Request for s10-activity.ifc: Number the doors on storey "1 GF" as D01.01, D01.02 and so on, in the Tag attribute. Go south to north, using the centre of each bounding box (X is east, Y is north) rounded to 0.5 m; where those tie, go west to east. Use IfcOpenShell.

First a look at what the model holds.

```python
import ifcopenshell
import ifcopenshell.util.element
import ifcopenshell.util.placement

model = ifcopenshell.open("s10-activity.ifc")
print(model.schema)
storey = next(s for s in model.by_type("IfcBuildingStorey") if s.Name == "1 GF")
doors = [e for e in ifcopenshell.util.element.get_decomposition(storey) if e.is_a("IfcDoor")]
for e in sorted(doors, key=lambda e: e.id()):
    origin = ifcopenshell.util.placement.get_local_placement(e.ObjectPlacement)[:3, 3]
    print(e.id(), e.Tag, e.Name, origin.round(2) + 0.0, sep=" | ")
```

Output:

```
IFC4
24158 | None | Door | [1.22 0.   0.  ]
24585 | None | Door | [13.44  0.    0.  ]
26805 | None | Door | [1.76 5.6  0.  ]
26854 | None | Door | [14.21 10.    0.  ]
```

```python
import ifcopenshell
import ifcopenshell.geom
import ifcopenshell.util.element
import ifcopenshell.util.shape

model = ifcopenshell.open("s10-activity.ifc")
settings = ifcopenshell.geom.settings()
settings.set("use-world-coords", True)


def centre(element):
    shape = ifcopenshell.geom.create_shape(settings, element)
    return ifcopenshell.util.shape.get_bbox_centroid(shape.geometry)


storey = next(s for s in model.by_type("IfcBuildingStorey") if s.Name == "1 GF")
doors = [e for e in ifcopenshell.util.element.get_decomposition(storey) if e.is_a("IfcDoor")]

# Insertion points can sit at a corner or the storey origin, so sort by the geometry (in metres).
centres = {e: centre(e) for e in doors}
doors.sort(key=lambda e: (round(centres[e][1] / 0.5), centres[e][0]))

for i, e in enumerate(doors, start=1):
    number = f"D01.{i:02d}"
    e.Tag = number
    print(e.id(), number)

model.write("s10-activity_v2.ifc")
```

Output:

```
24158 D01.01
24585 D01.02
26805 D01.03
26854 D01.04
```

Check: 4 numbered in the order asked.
